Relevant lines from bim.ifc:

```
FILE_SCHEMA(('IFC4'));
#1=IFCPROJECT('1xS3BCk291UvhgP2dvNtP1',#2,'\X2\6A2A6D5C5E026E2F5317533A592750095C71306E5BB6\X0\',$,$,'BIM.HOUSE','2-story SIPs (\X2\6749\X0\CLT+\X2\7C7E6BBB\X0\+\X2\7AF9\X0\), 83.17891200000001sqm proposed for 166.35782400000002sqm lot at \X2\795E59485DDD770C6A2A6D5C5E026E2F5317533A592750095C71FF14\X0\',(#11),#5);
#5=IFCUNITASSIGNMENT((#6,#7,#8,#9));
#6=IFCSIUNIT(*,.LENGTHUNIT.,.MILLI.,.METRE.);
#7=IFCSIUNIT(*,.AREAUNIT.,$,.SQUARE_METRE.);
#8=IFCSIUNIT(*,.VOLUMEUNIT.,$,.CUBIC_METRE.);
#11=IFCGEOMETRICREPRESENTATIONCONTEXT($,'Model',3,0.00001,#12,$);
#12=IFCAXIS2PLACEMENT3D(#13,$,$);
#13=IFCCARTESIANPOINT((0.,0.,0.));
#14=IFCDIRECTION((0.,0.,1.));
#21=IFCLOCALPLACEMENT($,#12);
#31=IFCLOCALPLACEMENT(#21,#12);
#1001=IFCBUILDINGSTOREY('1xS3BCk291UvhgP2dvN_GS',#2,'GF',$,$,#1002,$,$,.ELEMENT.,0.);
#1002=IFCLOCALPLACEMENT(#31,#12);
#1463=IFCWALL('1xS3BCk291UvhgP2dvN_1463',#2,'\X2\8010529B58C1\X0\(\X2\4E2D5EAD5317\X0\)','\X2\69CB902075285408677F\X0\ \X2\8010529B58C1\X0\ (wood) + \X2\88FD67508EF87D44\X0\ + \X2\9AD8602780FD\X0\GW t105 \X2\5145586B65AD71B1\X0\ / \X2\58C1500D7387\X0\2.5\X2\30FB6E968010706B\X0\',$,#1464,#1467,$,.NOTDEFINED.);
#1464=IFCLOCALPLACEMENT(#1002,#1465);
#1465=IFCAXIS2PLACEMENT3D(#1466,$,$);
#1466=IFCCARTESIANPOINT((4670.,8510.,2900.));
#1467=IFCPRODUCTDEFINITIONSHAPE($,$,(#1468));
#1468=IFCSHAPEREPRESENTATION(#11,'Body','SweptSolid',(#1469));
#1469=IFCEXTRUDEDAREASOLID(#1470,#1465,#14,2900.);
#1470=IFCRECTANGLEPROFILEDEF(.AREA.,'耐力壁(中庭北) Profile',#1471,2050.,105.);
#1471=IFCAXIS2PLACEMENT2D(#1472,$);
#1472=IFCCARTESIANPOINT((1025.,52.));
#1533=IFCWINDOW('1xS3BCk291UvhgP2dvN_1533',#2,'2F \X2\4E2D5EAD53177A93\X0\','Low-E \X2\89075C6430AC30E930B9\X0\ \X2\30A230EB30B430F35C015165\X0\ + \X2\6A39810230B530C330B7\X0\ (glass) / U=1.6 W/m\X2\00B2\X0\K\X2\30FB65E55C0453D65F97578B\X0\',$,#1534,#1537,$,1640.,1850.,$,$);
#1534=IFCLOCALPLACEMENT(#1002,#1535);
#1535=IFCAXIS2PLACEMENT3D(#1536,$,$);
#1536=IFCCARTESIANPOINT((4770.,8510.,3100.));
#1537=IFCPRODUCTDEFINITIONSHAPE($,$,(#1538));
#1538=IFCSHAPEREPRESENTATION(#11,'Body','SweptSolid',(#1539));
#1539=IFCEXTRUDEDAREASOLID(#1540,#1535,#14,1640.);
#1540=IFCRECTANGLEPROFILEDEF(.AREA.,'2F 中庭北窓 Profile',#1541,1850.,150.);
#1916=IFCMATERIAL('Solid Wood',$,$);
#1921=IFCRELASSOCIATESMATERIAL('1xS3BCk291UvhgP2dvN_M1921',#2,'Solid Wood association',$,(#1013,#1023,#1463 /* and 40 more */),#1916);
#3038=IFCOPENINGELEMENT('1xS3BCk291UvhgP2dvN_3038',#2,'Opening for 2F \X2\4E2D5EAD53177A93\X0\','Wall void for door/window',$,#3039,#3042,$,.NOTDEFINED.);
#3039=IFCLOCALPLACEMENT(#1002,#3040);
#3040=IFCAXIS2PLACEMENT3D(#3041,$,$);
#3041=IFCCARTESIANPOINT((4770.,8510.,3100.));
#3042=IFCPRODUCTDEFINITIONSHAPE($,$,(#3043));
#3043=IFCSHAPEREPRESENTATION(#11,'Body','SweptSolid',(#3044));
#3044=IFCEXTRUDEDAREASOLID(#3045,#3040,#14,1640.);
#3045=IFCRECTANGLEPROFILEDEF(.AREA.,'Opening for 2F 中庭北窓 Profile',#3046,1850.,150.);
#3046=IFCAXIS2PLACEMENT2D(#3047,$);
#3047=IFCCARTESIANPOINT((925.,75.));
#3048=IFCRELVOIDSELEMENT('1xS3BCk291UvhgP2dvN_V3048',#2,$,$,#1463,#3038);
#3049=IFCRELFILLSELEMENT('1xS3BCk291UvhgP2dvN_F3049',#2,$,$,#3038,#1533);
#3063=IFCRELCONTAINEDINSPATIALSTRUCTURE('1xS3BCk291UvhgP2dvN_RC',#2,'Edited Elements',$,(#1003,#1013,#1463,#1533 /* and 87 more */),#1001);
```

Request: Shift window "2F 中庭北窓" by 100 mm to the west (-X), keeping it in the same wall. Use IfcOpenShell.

```python
import ifcopenshell
import ifcopenshell.api.geometry
import ifcopenshell.util.placement

model = ifcopenshell.open("bim.ifc")

window = model.by_id(1533)
opening = window.FillsVoids[0].RelatingOpeningElement
wall = opening.VoidsElements[0].RelatingBuildingElement

wall_matrix = ifcopenshell.util.placement.get_local_placement(wall.ObjectPlacement)
shift = wall_matrix[:3, 0] * -100.0
before = ifcopenshell.util.placement.get_local_placement(window.ObjectPlacement)[:3, 3].copy()

# The window is not placed relative to its opening, so move both.
for product in (opening, window):
    matrix = ifcopenshell.util.placement.get_local_placement(product.ObjectPlacement)
    matrix[:3, 3] += shift
    ifcopenshell.api.geometry.edit_object_placement(model, product=product, matrix=matrix, is_si=False)

after = ifcopenshell.util.placement.get_local_placement(window.ObjectPlacement)[:3, 3]
print("window moved by", (after - before).round(3) + 0.0)

model.write("bim-out.ifc")
```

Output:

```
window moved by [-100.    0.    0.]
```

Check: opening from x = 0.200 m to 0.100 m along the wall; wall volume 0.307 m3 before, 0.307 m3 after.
